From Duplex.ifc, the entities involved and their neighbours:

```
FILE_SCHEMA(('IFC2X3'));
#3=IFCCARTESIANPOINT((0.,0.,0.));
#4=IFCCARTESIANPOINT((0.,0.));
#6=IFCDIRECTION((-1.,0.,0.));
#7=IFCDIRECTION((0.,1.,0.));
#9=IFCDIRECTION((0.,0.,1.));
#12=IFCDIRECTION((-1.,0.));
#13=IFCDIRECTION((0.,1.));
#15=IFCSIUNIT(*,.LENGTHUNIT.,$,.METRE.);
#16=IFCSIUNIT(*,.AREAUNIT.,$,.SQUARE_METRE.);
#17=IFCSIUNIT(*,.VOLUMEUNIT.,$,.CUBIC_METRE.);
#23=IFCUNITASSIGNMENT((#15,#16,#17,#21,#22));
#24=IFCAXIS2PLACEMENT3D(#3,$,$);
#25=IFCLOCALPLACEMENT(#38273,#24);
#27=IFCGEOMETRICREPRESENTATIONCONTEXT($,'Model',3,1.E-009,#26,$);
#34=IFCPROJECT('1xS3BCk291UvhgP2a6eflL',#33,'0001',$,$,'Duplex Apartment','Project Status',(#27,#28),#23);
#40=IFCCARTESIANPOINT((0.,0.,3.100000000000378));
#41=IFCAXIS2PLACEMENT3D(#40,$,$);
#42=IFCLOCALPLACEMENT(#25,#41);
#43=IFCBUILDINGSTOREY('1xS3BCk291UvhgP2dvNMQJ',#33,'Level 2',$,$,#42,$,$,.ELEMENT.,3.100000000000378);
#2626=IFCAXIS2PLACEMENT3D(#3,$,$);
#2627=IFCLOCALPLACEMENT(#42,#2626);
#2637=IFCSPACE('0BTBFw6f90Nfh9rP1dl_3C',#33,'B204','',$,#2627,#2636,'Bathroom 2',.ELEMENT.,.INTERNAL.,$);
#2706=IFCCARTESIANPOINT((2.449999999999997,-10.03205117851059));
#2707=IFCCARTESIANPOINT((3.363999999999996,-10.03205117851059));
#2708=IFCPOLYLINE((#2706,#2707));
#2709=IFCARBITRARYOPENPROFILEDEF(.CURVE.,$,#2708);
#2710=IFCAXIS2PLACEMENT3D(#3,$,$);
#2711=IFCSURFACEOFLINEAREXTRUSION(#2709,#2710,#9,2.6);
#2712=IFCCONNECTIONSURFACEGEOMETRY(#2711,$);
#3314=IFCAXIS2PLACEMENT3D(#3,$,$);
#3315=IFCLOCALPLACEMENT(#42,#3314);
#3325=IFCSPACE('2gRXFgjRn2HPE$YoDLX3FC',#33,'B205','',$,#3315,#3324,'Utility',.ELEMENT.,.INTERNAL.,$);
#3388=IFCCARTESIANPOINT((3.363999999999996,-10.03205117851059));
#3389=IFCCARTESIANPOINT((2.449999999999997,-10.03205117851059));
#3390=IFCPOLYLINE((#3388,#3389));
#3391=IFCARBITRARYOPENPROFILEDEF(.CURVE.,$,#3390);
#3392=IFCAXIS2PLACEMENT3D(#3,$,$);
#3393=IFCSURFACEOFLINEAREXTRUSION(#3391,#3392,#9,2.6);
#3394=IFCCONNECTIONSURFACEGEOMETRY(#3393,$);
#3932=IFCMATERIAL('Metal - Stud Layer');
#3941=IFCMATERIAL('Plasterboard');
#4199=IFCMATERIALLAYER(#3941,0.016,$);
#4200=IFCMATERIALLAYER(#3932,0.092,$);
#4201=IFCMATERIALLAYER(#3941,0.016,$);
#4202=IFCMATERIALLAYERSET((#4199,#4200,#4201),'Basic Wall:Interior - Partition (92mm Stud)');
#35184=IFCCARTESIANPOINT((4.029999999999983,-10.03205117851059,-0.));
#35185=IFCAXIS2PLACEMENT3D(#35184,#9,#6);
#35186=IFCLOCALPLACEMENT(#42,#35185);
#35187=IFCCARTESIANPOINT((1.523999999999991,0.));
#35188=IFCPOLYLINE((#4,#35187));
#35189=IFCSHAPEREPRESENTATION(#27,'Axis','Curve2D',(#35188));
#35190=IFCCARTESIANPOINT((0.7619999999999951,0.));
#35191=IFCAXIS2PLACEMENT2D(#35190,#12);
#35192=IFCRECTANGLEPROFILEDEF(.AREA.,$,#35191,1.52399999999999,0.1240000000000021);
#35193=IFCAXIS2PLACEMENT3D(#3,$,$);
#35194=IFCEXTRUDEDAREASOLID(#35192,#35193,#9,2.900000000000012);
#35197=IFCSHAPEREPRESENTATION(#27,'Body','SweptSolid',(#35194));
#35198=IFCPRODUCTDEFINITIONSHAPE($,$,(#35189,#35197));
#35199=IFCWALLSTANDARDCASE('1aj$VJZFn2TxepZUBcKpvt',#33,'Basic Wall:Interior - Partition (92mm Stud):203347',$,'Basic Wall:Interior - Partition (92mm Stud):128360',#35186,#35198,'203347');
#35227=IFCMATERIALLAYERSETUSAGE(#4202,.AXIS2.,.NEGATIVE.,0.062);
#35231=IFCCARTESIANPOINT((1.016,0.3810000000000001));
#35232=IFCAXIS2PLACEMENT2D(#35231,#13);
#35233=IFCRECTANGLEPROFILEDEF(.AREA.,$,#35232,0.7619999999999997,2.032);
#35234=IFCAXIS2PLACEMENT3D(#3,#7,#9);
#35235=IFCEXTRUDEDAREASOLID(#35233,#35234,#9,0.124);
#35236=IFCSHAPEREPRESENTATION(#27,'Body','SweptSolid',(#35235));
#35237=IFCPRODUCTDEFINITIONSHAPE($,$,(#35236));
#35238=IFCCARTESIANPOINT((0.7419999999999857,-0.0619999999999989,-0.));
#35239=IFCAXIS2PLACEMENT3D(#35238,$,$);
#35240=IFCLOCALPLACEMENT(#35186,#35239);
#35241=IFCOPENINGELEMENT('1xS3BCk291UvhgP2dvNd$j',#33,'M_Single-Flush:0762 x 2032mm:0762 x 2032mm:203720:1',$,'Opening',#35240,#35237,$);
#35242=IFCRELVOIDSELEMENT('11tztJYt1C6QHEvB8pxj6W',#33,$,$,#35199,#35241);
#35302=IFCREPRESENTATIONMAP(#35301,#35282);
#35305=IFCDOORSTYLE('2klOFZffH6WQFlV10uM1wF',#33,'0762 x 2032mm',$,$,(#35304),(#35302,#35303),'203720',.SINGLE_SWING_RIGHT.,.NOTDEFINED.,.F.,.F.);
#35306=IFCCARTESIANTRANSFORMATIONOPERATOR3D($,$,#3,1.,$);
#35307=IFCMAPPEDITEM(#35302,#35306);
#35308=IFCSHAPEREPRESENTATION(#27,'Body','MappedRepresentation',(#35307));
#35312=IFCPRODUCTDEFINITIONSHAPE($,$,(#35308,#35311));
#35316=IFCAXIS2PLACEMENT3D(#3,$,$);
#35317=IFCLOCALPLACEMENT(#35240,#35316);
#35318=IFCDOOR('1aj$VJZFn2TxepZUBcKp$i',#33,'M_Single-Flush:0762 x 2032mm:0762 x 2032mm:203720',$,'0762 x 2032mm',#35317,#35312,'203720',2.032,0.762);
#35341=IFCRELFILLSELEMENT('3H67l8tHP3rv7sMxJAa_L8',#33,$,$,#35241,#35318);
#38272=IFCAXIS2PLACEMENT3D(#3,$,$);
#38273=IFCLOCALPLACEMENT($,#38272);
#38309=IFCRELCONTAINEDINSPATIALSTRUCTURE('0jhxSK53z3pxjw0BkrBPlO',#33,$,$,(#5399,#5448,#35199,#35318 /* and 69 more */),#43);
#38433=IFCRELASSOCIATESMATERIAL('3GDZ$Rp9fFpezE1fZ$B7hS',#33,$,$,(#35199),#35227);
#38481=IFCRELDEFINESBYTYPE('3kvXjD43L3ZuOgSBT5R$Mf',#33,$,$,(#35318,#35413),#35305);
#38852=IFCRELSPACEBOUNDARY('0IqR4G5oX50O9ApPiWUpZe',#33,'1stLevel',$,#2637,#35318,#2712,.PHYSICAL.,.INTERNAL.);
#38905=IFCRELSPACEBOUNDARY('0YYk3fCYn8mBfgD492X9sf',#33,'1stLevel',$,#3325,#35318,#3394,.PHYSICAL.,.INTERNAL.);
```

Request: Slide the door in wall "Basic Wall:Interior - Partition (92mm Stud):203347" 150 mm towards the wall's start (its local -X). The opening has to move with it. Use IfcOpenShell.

```python
import numpy as np
import ifcopenshell
import ifcopenshell.api.geometry
import ifcopenshell.util.placement
import ifcopenshell.util.unit

model = ifcopenshell.open("Duplex.ifc")
unit_scale = ifcopenshell.util.unit.calculate_unit_scale(model)

door = model.by_guid("1aj$VJZFn2TxepZUBcKp$i")
opening = door.FillsVoids[0].RelatingOpeningElement
wall = opening.VoidsElements[0].RelatingBuildingElement

wall_matrix = ifcopenshell.util.placement.get_local_placement(wall.ObjectPlacement)
shift = wall_matrix[:3, 0] * -0.15 / unit_scale
before = ifcopenshell.util.placement.get_local_placement(door.ObjectPlacement)[:3, 3].copy()

# The door is placed relative to its opening, so it follows when the opening moves.
matrix = ifcopenshell.util.placement.get_local_placement(opening.ObjectPlacement)
matrix[:3, 3] += shift
ifcopenshell.api.geometry.edit_object_placement(
    model, product=opening, matrix=matrix, is_si=False, should_transform_children=True
)

# Space boundary surfaces are stored in each space's coordinates; move them too.
for rel in door.ProvidesBoundaries:
    if not rel.ConnectionGeometry:
        continue
    surface = rel.ConnectionGeometry.SurfaceOnRelatingElement
    space_matrix = ifcopenshell.util.placement.get_local_placement(rel.RelatingSpace.ObjectPlacement)
    point = np.array(surface.Position.Location.Coordinates) + space_matrix[:3, :3].T @ shift
    surface.Position = model.createIfcAxis2Placement3D(
        model.createIfcCartesianPoint(point.tolist()), surface.Position.Axis, surface.Position.RefDirection
    )

after = ifcopenshell.util.placement.get_local_placement(door.ObjectPlacement)[:3, 3]
print("door moved by", (after - before).round(3) + 0.0)

model.write("Duplex-out.ifc")
```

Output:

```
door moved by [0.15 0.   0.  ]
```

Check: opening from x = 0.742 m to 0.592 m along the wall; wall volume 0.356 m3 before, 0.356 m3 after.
